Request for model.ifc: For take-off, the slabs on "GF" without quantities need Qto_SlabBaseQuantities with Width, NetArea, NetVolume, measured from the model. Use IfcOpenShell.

First a look at what the model holds.

```python
import ifcopenshell
import ifcopenshell.util.element
import ifcopenshell.util.unit

model = ifcopenshell.open("model.ifc")
print(model.schema)
for unit_type in ("LENGTHUNIT", "AREAUNIT", "VOLUMEUNIT"):
    print(unit_type, ifcopenshell.util.unit.calculate_unit_scale(model, unit_type))
storey = next(s for s in model.by_type("IfcBuildingStorey") if s.Name == "GF")
slabs = [e for e in ifcopenshell.util.element.get_decomposition(storey) if e.is_a("IfcSlab")]
for e in sorted(slabs, key=lambda e: e.id()):
    print(e.id(), e.is_a(), e.Name, list(ifcopenshell.util.element.get_psets(e, qtos_only=True)), sep=" | ")
```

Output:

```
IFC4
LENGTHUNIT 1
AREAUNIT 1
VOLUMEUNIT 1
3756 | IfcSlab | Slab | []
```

```python
import ifcopenshell
import ifcopenshell.api.pset
import ifcopenshell.geom
import ifcopenshell.util.element
import ifcopenshell.util.shape
import ifcopenshell.util.unit

model = ifcopenshell.open("model.ifc")
unit_scale = ifcopenshell.util.unit.calculate_unit_scale(model)
area_scale = ifcopenshell.util.unit.calculate_unit_scale(model, "AREAUNIT")
volume_scale = ifcopenshell.util.unit.calculate_unit_scale(model, "VOLUMEUNIT")
settings = ifcopenshell.geom.settings()

storey = next(s for s in model.by_type("IfcBuildingStorey") if s.Name == "GF")
slabs = [e for e in ifcopenshell.util.element.get_decomposition(storey) if e.is_a("IfcSlab")]

for e in sorted(slabs, key=lambda e: e.id()):
    if ifcopenshell.util.element.get_psets(e, qtos_only=True, should_inherit=False):
        continue
    # Geometry comes back in metres, in the element's own axes.
    shape = ifcopenshell.geom.create_shape(settings, e)
    values = {
        "Width": ifcopenshell.util.shape.get_z(shape.geometry) / unit_scale,
        "NetArea": ifcopenshell.util.shape.get_footprint_area(shape.geometry) / area_scale,
        "NetVolume": ifcopenshell.util.shape.get_volume(shape.geometry) / volume_scale,
    }
    qto = ifcopenshell.api.pset.add_qto(model, product=e, name="Qto_SlabBaseQuantities")
    ifcopenshell.api.pset.edit_qto(model, qto=qto, properties=values)
    print(e.id(), {k: round(v, 3) for k, v in values.items()})

model.write("model_edited.ifc")
```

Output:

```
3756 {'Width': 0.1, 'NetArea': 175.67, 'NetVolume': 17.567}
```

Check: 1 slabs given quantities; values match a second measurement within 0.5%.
